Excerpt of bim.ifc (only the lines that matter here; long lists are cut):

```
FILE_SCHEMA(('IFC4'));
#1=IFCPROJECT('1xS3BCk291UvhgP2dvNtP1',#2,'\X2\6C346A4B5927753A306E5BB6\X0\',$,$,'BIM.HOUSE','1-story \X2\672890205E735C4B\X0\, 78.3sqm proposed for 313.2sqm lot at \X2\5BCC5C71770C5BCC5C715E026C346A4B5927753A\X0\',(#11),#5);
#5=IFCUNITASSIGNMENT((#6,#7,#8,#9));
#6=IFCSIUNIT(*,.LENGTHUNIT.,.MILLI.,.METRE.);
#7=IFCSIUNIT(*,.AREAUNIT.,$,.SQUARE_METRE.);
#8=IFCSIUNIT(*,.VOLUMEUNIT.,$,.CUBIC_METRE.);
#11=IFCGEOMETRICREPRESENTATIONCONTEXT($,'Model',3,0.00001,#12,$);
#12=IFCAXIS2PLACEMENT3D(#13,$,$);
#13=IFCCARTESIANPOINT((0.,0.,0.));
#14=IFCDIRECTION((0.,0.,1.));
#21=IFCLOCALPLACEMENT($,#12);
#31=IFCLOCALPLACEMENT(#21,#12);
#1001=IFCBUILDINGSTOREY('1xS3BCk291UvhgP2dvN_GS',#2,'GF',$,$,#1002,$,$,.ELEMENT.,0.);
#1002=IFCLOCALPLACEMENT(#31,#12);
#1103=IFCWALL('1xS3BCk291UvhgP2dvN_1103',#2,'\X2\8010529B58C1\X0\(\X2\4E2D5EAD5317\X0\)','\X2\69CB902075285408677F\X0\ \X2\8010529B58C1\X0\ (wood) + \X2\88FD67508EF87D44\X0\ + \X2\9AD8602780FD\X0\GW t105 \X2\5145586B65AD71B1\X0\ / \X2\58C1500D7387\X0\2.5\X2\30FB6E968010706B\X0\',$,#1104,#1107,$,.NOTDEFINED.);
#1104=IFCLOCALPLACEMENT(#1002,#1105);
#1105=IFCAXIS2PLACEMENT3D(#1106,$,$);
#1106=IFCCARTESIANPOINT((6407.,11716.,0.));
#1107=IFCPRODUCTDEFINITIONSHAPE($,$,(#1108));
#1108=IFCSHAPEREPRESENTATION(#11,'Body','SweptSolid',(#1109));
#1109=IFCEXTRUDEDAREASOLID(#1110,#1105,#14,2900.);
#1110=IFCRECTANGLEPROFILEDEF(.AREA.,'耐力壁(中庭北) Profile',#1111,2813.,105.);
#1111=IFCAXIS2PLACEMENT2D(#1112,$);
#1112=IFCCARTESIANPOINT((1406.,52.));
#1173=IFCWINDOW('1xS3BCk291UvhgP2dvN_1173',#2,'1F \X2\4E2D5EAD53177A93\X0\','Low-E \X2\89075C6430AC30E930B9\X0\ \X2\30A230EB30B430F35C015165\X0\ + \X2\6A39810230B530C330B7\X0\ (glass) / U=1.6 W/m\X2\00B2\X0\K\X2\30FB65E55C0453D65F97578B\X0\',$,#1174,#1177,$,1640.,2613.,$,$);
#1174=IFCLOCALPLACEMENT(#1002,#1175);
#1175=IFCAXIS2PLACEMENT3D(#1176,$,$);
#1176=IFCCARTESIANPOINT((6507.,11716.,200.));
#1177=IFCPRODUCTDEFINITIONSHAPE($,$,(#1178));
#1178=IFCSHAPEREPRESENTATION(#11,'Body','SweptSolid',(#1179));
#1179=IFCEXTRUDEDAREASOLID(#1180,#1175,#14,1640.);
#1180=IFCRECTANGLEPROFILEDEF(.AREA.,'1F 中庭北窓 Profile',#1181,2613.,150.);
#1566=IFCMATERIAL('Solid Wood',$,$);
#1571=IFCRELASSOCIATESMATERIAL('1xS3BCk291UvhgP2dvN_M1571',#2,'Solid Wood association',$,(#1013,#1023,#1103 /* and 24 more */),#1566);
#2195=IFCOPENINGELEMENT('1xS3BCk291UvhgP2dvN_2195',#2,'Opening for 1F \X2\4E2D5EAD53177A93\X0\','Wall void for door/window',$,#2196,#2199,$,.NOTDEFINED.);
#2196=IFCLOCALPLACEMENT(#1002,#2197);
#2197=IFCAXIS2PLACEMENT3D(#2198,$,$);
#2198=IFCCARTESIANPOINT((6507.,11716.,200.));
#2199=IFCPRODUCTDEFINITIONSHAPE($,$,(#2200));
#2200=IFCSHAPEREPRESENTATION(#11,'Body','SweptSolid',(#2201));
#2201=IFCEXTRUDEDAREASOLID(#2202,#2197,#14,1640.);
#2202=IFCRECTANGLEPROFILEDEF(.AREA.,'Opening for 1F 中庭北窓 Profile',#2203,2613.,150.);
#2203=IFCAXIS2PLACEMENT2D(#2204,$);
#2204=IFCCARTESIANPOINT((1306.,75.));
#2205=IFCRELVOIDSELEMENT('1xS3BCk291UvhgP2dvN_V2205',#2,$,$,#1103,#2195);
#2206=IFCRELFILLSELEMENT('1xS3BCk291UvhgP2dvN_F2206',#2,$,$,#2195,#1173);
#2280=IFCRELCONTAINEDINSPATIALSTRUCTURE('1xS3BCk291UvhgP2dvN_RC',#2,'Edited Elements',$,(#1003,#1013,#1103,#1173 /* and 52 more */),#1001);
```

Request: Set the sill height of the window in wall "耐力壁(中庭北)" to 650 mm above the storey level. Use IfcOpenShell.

```python
import numpy as np
import ifcopenshell
import ifcopenshell.api.geometry
import ifcopenshell.geom
import ifcopenshell.util.element
import ifcopenshell.util.placement
import ifcopenshell.util.shape
import ifcopenshell.util.unit

model = ifcopenshell.open("bim.ifc")
unit_scale = ifcopenshell.util.unit.calculate_unit_scale(model)

window = model.by_id(1173)
opening = window.FillsVoids[0].RelatingOpeningElement
storey = ifcopenshell.util.element.get_container(window, ifc_class="IfcBuildingStorey")
level = ifcopenshell.util.placement.get_local_placement(storey.ObjectPlacement)[2, 3]

# The opening's origin need not be at the sill, so measure its lowest point.
shape = ifcopenshell.geom.create_shape(ifcopenshell.geom.settings(), opening)
bottom = ifcopenshell.util.shape.get_shape_bottom_elevation(shape, shape.geometry) / unit_scale
dz = level + 650.0 - bottom

shift = np.array([0.0, 0.0, dz])
# The window is not placed relative to its opening, so move both.
for product in (opening, window):
    matrix = ifcopenshell.util.placement.get_local_placement(product.ObjectPlacement)
    matrix[:3, 3] += shift
    ifcopenshell.api.geometry.edit_object_placement(model, product=product, matrix=matrix, is_si=False)

print(f"moved by {dz * unit_scale:+.3f} m")

model.write("bim-out.ifc")
```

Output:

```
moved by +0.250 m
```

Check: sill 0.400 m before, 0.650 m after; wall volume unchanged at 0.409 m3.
